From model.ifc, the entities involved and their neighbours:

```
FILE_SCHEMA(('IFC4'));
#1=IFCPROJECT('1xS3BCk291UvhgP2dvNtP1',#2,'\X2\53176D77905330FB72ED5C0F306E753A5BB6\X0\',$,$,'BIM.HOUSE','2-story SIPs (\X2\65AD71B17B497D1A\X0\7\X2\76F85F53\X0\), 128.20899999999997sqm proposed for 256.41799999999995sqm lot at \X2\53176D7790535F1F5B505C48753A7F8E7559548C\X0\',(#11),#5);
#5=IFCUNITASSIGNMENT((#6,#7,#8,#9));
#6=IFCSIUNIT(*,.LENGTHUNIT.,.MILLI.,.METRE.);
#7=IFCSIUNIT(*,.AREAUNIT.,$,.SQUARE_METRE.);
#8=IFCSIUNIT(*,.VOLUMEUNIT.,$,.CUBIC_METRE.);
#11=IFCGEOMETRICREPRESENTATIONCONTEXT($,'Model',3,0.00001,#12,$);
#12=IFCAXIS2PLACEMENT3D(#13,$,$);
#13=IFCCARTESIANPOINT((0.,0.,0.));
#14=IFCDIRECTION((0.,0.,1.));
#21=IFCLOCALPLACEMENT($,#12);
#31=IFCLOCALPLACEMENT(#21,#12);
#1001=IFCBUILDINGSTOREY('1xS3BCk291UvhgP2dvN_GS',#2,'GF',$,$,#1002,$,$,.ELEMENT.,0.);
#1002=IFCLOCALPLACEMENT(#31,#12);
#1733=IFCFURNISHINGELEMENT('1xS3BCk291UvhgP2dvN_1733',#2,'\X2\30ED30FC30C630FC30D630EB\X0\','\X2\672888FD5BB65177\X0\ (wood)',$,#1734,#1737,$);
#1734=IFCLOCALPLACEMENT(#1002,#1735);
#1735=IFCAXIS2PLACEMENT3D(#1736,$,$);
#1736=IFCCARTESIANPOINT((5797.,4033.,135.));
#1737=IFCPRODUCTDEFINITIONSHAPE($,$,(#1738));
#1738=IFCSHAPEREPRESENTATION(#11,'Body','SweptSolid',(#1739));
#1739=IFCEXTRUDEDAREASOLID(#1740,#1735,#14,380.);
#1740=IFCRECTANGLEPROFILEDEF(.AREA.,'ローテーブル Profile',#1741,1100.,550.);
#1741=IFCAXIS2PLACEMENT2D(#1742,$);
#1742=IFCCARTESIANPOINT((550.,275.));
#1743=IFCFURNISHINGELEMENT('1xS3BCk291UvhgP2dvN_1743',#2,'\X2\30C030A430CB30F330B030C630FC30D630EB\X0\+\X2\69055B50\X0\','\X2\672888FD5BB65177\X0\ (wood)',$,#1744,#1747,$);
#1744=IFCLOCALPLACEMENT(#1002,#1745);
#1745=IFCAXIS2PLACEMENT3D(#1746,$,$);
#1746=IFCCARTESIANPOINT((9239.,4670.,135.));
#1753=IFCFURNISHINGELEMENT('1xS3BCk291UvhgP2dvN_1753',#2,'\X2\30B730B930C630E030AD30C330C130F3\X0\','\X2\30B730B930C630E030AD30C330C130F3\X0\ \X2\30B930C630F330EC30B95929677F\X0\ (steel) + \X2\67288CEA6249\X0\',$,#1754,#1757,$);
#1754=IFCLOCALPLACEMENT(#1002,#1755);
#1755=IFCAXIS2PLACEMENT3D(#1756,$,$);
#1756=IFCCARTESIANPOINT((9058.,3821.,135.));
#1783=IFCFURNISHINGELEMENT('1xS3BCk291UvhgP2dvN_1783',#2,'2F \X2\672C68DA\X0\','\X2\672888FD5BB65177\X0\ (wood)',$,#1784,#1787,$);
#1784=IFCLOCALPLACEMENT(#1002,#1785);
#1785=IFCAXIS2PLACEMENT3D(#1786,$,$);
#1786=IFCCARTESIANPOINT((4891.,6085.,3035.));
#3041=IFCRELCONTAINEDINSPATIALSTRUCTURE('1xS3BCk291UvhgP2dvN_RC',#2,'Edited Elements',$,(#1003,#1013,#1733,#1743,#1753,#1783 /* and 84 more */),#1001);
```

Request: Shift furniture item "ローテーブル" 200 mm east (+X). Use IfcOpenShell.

```python
import ifcopenshell
import ifcopenshell.api.geometry
import ifcopenshell.util.placement
import ifcopenshell.util.unit

model = ifcopenshell.open("model.ifc")
unit_scale = ifcopenshell.util.unit.calculate_unit_scale(model)

item = model.by_guid("1xS3BCk291UvhgP2dvN_1733")
matrix = ifcopenshell.util.placement.get_local_placement(item.ObjectPlacement)
matrix[0, 3] += 0.2 / unit_scale
ifcopenshell.api.geometry.edit_object_placement(model, product=item, matrix=matrix, is_si=False)

print(ifcopenshell.util.placement.get_local_placement(item.ObjectPlacement).round(3) + 0.0)

model.write("model-out.ifc")
```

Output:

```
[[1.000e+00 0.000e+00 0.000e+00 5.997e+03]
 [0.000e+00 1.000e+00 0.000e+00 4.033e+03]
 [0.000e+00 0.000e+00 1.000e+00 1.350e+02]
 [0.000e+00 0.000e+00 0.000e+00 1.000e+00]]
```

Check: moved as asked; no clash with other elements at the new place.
